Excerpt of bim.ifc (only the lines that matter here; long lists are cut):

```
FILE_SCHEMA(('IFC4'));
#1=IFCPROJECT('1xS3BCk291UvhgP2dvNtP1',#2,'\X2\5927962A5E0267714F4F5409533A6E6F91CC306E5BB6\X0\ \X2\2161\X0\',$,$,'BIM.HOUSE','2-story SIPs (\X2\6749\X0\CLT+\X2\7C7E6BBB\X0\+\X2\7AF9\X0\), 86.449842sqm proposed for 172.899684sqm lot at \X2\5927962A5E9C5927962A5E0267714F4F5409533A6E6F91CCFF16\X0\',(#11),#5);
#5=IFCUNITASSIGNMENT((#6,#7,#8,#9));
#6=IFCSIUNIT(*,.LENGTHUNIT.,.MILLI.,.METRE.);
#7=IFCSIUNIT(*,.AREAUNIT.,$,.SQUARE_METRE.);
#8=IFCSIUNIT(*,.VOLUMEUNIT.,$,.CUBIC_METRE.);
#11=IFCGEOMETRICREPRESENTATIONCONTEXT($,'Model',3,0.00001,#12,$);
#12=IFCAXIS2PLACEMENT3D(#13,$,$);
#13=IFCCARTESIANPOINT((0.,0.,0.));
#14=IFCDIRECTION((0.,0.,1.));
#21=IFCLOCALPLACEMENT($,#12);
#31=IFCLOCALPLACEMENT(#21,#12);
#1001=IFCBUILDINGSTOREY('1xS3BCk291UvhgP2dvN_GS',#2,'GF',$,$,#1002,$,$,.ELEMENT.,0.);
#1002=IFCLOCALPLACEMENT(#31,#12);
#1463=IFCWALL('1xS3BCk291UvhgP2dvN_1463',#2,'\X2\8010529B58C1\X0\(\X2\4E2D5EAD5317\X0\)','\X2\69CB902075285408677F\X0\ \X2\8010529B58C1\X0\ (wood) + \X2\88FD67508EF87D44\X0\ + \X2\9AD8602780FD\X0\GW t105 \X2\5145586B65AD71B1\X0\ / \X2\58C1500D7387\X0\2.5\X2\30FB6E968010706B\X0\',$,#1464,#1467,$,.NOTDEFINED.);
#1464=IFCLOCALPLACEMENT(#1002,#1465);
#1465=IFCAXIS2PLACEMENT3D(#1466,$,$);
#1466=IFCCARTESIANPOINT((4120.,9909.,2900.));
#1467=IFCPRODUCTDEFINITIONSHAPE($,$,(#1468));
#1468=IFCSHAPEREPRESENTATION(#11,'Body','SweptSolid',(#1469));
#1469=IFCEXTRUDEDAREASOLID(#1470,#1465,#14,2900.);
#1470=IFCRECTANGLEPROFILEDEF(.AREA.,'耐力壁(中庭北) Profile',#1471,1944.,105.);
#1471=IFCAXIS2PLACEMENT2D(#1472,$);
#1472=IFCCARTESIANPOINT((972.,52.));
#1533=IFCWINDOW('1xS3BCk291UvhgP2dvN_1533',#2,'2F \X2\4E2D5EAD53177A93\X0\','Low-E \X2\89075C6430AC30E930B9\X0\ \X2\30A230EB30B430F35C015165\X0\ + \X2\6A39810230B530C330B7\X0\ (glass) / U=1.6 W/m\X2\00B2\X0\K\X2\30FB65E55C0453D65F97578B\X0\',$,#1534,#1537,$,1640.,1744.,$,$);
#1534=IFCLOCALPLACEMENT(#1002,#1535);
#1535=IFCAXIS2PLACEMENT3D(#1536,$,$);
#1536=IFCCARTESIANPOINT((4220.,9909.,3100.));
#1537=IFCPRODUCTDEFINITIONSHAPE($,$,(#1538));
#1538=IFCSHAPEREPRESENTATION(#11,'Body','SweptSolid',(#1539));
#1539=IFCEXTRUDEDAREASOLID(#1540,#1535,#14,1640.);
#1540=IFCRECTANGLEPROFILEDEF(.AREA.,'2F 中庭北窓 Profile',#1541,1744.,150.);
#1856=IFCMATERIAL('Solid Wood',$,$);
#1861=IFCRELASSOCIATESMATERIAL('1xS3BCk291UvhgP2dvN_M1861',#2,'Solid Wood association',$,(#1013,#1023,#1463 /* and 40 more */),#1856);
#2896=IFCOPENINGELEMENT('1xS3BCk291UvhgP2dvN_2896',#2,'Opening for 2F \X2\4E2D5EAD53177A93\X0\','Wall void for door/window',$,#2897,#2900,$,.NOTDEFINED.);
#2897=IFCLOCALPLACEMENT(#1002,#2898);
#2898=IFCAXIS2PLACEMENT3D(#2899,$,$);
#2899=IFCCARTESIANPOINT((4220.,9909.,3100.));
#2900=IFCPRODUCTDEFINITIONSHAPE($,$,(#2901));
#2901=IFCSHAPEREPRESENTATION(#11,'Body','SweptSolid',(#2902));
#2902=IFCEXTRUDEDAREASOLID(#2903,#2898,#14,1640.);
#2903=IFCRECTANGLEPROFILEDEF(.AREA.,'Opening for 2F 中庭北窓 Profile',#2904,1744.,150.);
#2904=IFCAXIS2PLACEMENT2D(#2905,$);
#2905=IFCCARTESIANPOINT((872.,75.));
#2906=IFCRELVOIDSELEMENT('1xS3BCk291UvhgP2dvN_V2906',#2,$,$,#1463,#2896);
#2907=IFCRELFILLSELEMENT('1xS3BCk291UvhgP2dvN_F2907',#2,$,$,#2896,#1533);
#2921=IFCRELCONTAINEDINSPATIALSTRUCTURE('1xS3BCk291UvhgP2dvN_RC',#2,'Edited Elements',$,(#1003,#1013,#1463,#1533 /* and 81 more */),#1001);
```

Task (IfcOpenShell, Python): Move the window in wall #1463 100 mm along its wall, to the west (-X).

```python
import ifcopenshell
import ifcopenshell.api.geometry
import ifcopenshell.util.placement

model = ifcopenshell.open("bim.ifc")

window = model.by_id(1533)
opening = window.FillsVoids[0].RelatingOpeningElement
wall = opening.VoidsElements[0].RelatingBuildingElement

wall_matrix = ifcopenshell.util.placement.get_local_placement(wall.ObjectPlacement)
shift = wall_matrix[:3, 0] * -100.0
before = ifcopenshell.util.placement.get_local_placement(window.ObjectPlacement)[:3, 3].copy()

# The window is not placed relative to its opening, so move both.
for product in (opening, window):
    matrix = ifcopenshell.util.placement.get_local_placement(product.ObjectPlacement)
    matrix[:3, 3] += shift
    ifcopenshell.api.geometry.edit_object_placement(model, product=product, matrix=matrix, is_si=False)

after = ifcopenshell.util.placement.get_local_placement(window.ObjectPlacement)[:3, 3]
print("window moved by", (after - before).round(3) + 0.0)

model.write("bim-out.ifc")
```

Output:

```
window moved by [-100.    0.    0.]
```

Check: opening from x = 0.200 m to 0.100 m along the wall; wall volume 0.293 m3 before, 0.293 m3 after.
